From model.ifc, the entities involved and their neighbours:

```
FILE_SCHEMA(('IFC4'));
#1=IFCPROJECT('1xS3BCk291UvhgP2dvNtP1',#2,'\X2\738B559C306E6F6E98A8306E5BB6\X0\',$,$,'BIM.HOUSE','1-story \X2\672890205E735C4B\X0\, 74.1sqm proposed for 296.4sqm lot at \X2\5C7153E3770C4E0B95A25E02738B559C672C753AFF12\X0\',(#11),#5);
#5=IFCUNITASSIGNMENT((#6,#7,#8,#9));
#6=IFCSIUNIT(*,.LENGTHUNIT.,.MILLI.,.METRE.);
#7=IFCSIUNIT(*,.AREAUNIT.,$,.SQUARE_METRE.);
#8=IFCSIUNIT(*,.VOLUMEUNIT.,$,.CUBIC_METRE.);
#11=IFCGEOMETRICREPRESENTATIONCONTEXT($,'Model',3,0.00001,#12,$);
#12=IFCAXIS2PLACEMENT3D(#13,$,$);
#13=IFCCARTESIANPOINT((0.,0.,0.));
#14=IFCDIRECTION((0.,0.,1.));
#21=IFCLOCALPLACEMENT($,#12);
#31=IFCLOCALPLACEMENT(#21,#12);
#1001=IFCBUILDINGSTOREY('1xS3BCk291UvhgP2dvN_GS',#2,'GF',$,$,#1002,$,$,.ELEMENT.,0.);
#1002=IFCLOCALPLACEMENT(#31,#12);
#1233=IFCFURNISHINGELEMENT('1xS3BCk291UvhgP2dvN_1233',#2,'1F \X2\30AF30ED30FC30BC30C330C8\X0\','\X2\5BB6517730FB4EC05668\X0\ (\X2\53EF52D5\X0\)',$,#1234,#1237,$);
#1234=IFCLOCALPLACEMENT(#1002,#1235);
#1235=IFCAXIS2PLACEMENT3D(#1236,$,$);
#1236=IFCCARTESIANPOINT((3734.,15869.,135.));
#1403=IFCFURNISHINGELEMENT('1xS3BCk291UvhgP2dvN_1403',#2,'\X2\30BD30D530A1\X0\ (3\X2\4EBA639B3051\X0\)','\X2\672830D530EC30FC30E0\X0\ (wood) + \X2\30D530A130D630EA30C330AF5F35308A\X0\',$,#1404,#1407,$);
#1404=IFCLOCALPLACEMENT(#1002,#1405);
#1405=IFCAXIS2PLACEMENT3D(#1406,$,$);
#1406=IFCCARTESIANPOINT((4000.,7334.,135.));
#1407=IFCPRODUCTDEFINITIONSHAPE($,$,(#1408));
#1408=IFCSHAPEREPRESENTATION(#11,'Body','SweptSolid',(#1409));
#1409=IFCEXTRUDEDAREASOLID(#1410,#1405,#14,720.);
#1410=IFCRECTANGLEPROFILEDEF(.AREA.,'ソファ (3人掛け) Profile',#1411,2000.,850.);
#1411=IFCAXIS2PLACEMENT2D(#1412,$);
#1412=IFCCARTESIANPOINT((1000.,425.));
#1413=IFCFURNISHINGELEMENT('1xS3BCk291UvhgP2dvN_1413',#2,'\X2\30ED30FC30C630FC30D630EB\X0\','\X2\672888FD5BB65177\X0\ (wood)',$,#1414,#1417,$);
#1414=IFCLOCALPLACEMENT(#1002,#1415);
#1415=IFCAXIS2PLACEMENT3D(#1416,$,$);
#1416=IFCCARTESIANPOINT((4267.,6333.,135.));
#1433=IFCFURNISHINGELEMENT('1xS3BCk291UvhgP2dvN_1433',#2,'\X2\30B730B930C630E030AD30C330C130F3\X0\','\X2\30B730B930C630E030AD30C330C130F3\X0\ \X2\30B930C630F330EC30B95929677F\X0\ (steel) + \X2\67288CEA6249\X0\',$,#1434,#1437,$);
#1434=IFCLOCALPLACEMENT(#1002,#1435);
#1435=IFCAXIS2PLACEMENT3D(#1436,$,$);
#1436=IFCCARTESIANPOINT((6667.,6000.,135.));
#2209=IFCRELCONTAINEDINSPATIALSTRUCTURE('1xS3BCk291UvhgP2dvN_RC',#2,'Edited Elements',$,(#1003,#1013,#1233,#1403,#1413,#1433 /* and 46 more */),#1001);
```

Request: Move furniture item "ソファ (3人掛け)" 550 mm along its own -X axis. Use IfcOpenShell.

```python
import ifcopenshell
import ifcopenshell.api.geometry
import ifcopenshell.util.placement
import ifcopenshell.util.unit

model = ifcopenshell.open("model.ifc")
unit_scale = ifcopenshell.util.unit.calculate_unit_scale(model)

item = model.by_guid("1xS3BCk291UvhgP2dvN_1403")
matrix = ifcopenshell.util.placement.get_local_placement(item.ObjectPlacement)
matrix[:3, 3] -= matrix[:3, 0] * 0.55 / unit_scale
ifcopenshell.api.geometry.edit_object_placement(model, product=item, matrix=matrix, is_si=False)

print(ifcopenshell.util.placement.get_local_placement(item.ObjectPlacement).round(3) + 0.0)

model.write("model_rev.ifc")
```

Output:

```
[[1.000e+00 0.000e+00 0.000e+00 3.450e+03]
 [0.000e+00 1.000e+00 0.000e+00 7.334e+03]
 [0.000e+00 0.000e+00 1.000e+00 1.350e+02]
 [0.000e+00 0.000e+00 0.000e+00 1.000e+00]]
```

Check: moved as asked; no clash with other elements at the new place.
